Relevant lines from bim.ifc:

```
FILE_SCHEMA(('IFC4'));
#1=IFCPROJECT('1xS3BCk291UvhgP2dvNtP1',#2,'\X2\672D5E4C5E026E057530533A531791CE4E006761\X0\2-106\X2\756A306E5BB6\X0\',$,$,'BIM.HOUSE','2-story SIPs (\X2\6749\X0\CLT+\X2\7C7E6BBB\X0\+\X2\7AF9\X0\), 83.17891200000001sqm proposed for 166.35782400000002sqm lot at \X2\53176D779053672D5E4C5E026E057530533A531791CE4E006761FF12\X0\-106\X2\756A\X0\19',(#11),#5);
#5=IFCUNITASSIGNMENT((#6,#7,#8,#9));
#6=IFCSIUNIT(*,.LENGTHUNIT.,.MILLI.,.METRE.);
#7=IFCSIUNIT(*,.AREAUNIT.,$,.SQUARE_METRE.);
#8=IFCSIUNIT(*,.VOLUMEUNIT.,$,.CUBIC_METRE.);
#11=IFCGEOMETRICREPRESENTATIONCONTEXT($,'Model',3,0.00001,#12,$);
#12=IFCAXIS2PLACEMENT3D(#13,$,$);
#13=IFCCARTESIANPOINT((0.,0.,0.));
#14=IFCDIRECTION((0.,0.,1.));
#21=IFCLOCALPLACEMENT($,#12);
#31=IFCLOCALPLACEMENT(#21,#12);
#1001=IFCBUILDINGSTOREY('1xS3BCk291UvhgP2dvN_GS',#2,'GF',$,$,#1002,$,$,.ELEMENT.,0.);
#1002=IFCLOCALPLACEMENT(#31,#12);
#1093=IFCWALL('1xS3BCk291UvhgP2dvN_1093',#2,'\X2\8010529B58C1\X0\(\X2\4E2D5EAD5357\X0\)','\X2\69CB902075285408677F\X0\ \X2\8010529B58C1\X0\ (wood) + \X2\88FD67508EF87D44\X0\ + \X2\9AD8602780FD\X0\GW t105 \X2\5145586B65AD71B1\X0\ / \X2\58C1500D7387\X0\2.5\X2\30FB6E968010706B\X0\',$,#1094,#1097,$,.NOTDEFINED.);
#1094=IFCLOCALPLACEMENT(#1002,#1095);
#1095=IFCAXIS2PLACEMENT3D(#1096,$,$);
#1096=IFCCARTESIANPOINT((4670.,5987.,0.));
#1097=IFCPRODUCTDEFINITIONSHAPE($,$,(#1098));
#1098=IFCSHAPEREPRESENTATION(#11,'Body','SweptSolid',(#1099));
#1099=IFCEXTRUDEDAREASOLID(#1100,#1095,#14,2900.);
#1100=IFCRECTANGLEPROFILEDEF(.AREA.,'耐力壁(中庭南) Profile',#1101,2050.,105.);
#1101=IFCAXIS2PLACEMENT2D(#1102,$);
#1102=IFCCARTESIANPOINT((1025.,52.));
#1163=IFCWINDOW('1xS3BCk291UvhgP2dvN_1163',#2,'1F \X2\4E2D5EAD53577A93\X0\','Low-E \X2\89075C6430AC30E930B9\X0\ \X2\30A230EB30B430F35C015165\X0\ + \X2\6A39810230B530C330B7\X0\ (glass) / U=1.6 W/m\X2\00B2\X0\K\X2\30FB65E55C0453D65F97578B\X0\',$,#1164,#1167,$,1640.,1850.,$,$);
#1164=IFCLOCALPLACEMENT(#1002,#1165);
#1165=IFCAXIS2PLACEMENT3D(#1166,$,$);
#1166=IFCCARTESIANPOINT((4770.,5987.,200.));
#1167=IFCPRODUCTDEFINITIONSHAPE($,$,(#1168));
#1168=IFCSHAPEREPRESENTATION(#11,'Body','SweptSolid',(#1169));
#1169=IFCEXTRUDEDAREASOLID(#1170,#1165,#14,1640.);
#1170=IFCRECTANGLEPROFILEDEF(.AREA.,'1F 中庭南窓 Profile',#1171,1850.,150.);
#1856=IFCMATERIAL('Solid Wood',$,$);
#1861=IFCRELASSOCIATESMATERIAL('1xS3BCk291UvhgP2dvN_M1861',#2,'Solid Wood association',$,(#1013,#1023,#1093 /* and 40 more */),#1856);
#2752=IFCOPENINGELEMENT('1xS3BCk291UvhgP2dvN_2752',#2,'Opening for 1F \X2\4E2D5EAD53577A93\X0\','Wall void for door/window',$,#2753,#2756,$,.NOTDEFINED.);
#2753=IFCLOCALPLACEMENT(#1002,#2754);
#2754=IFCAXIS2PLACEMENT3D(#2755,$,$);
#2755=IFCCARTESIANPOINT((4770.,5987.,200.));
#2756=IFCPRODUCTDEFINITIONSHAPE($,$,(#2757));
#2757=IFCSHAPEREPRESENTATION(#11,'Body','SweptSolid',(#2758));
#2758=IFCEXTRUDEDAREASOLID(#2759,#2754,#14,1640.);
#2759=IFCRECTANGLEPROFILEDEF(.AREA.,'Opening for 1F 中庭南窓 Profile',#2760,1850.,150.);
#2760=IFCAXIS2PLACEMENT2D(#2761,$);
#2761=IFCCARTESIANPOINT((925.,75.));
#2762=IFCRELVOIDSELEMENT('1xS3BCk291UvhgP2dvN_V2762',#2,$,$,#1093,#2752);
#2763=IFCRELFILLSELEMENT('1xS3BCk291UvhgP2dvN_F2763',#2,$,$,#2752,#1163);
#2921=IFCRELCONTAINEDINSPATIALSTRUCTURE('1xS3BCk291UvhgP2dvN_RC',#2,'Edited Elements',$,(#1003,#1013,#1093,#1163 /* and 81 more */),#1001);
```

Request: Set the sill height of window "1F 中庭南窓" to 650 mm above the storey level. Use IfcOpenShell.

```python
import numpy as np
import ifcopenshell
import ifcopenshell.api.geometry
import ifcopenshell.geom
import ifcopenshell.util.element
import ifcopenshell.util.placement
import ifcopenshell.util.shape
import ifcopenshell.util.unit

model = ifcopenshell.open("bim.ifc")
unit_scale = ifcopenshell.util.unit.calculate_unit_scale(model)

window = model.by_guid("1xS3BCk291UvhgP2dvN_1163")
opening = window.FillsVoids[0].RelatingOpeningElement
storey = ifcopenshell.util.element.get_container(window, ifc_class="IfcBuildingStorey")
level = ifcopenshell.util.placement.get_local_placement(storey.ObjectPlacement)[2, 3]

# The opening's origin need not be at the sill, so measure its lowest point.
shape = ifcopenshell.geom.create_shape(ifcopenshell.geom.settings(), opening)
bottom = ifcopenshell.util.shape.get_shape_bottom_elevation(shape, shape.geometry) / unit_scale
dz = level + 0.65 / unit_scale - bottom

shift = np.array([0.0, 0.0, dz])
# The window is not placed relative to its opening, so move both.
for product in (opening, window):
    matrix = ifcopenshell.util.placement.get_local_placement(product.ObjectPlacement)
    matrix[:3, 3] += shift
    ifcopenshell.api.geometry.edit_object_placement(model, product=product, matrix=matrix, is_si=False)

print(f"moved by {dz * unit_scale:+.3f} m")

model.write("bim_edited.ifc")
```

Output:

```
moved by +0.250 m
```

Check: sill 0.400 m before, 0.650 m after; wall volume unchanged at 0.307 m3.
